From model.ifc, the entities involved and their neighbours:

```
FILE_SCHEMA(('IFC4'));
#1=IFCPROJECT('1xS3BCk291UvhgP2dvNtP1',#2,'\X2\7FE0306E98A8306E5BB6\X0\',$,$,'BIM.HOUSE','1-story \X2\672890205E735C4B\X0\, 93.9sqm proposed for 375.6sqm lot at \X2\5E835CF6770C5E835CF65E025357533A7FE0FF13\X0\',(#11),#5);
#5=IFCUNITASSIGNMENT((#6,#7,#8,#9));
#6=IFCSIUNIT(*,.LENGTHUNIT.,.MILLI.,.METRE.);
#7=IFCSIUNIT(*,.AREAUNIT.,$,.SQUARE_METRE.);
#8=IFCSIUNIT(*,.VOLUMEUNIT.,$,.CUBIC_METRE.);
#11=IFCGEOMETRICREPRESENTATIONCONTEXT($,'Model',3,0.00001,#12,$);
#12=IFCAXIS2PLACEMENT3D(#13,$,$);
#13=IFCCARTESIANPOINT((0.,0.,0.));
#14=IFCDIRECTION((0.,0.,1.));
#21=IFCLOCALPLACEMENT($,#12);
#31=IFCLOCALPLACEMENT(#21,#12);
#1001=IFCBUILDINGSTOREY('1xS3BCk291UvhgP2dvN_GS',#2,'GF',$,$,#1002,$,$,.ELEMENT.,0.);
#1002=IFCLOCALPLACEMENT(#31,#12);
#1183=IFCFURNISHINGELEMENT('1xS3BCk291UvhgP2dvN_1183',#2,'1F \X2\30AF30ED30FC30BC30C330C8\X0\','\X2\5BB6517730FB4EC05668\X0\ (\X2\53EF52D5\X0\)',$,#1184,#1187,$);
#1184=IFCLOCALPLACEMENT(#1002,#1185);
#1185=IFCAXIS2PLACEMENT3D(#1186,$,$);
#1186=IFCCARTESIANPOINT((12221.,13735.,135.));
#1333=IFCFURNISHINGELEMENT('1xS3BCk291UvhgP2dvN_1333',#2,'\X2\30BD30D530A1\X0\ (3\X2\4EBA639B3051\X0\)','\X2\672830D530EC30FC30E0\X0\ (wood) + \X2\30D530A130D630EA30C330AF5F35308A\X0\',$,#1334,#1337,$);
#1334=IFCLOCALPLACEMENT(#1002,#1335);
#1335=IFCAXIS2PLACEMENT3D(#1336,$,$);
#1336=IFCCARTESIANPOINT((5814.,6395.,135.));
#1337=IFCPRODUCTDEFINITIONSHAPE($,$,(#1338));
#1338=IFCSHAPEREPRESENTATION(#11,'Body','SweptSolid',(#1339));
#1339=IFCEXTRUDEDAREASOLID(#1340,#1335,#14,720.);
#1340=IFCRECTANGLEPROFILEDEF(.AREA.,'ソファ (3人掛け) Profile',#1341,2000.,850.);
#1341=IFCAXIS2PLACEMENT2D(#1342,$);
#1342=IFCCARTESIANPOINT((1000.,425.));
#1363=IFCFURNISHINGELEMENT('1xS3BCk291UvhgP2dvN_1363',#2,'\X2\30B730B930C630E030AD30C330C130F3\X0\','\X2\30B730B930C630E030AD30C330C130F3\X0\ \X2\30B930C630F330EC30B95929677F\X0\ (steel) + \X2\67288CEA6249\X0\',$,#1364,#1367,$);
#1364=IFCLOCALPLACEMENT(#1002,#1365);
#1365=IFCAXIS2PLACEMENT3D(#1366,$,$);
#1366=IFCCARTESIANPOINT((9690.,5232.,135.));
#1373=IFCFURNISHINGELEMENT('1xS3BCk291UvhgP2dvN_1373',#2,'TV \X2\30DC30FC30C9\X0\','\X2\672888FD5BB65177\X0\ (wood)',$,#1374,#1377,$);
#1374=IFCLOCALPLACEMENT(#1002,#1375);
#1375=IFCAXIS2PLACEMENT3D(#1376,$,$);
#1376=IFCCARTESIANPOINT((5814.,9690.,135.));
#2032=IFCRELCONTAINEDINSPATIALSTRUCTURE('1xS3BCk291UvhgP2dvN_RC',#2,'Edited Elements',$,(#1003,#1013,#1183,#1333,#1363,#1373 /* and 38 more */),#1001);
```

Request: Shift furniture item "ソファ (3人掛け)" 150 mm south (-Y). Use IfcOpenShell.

```python
import ifcopenshell
import ifcopenshell.api.geometry
import ifcopenshell.util.placement
import ifcopenshell.util.unit

model = ifcopenshell.open("model.ifc")
unit_scale = ifcopenshell.util.unit.calculate_unit_scale(model)

item = model.by_id(1333)
matrix = ifcopenshell.util.placement.get_local_placement(item.ObjectPlacement)
matrix[1, 3] -= 0.15 / unit_scale
ifcopenshell.api.geometry.edit_object_placement(model, product=item, matrix=matrix, is_si=False)

print(ifcopenshell.util.placement.get_local_placement(item.ObjectPlacement).round(3) + 0.0)

model.write("model_edited.ifc")
```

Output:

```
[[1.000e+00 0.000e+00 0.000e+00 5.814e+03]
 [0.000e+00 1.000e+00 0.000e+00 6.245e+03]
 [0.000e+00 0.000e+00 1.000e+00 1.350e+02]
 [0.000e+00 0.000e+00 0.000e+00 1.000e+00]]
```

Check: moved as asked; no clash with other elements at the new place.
